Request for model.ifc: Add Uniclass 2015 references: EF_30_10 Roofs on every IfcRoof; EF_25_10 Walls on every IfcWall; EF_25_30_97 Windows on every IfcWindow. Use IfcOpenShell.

First a look at what the model holds.

```python
import ifcopenshell

model = ifcopenshell.open("model.ifc")
print(model.schema)
print("classifications:", [c.Name for c in model.by_type("IfcClassification")])
for ifc_class in ("IfcDoor", "IfcRoof", "IfcStair", "IfcWall", "IfcWindow"):
    print(ifc_class, len(model.by_type(ifc_class)))
```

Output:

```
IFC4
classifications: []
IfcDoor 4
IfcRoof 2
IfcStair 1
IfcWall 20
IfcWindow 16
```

```python
import ifcopenshell
import ifcopenshell.api.classification

model = ifcopenshell.open("model.ifc")

system = ifcopenshell.api.classification.add_classification(model, classification="Uniclass 2015")

codes = {
    "IfcRoof": ("EF_30_10", "Roofs"),
    "IfcWall": ("EF_25_10", "Walls"),
    "IfcWindow": ("EF_25_30_97", "Windows"),
}
for ifc_class, (code, name) in codes.items():
    products = model.by_type(ifc_class)
    ifcopenshell.api.classification.add_reference(
        model, products=products, classification=system, identification=code, name=name
    )
    print(code, len(products))

model.write("model_v2.ifc")
```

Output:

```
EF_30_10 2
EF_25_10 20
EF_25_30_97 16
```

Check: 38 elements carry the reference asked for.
